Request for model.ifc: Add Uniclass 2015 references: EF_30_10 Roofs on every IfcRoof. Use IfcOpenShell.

First a look at what the model holds.

```python
import ifcopenshell

model = ifcopenshell.open("model.ifc")
print(model.schema)
print("classifications:", [c.Name for c in model.by_type("IfcClassification")])
for ifc_class in ("IfcDoor", "IfcRoof", "IfcStair", "IfcWall", "IfcWindow"):
    print(ifc_class, len(model.by_type(ifc_class)))
```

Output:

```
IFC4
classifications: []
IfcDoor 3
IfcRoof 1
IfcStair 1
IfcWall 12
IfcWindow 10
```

```python
import ifcopenshell
import ifcopenshell.api.classification

model = ifcopenshell.open("model.ifc")

system = ifcopenshell.api.classification.add_classification(model, classification="Uniclass 2015")

codes = {
    "IfcRoof": ("EF_30_10", "Roofs"),
}
for ifc_class, (code, name) in codes.items():
    products = model.by_type(ifc_class)
    ifcopenshell.api.classification.add_reference(
        model, products=products, classification=system, identification=code, name=name
    )
    print(code, len(products))

model.write("model_updated.ifc")
```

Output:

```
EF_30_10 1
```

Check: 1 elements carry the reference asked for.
